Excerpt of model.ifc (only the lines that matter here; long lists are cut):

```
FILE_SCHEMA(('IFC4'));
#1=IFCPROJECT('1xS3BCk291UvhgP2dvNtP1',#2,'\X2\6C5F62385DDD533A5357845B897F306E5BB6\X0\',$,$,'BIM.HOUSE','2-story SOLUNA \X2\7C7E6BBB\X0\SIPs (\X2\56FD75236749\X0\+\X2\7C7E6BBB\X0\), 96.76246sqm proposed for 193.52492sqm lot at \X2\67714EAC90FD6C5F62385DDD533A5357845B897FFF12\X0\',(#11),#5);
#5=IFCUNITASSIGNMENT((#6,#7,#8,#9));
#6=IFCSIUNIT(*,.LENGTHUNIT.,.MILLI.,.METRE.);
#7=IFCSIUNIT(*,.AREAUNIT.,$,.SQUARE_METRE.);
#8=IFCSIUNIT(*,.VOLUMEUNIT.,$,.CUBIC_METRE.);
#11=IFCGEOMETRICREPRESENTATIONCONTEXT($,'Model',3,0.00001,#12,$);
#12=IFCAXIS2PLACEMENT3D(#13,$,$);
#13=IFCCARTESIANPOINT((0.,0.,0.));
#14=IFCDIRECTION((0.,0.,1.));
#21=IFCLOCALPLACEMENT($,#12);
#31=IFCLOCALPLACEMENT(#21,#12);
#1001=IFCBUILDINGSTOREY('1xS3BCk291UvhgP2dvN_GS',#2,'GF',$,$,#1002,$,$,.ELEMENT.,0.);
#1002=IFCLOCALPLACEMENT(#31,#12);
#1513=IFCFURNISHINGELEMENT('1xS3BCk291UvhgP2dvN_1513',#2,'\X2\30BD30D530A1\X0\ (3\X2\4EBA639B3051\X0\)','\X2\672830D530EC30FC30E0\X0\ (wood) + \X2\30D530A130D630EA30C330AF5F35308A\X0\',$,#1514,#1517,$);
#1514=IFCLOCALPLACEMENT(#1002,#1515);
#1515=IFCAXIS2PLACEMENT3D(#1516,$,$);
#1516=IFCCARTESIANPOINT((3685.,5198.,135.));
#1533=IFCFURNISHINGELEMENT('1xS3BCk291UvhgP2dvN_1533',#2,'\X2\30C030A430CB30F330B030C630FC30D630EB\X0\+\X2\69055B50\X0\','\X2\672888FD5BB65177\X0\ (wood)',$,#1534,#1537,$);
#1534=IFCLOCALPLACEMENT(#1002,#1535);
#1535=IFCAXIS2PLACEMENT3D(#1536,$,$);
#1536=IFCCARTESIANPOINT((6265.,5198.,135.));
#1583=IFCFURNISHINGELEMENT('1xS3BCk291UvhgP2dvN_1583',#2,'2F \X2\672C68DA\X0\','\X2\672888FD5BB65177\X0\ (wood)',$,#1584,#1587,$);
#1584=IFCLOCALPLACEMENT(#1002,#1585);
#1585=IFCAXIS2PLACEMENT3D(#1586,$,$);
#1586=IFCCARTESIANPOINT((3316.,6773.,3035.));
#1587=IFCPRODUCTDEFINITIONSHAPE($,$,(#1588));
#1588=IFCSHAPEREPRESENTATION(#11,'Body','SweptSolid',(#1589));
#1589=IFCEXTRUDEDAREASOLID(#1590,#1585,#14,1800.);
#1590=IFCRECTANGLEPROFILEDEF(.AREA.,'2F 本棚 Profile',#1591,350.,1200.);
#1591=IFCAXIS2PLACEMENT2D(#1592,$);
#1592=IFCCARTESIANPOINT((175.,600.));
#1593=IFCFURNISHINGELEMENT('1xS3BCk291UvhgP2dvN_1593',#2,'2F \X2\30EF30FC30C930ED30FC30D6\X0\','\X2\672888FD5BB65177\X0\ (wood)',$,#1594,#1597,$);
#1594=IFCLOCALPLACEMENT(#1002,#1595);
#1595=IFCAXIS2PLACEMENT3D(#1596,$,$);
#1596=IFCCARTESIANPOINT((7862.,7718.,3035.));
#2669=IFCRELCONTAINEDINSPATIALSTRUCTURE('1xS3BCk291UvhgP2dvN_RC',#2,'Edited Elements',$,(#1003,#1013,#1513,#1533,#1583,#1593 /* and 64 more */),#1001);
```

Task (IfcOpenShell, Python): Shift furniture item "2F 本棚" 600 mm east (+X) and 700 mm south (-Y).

```python
import ifcopenshell
import ifcopenshell.api.geometry
import ifcopenshell.util.placement

model = ifcopenshell.open("model.ifc")

item = model.by_id(1583)
matrix = ifcopenshell.util.placement.get_local_placement(item.ObjectPlacement)
matrix[0, 3] += 600.0
matrix[1, 3] -= 700.0
ifcopenshell.api.geometry.edit_object_placement(model, product=item, matrix=matrix, is_si=False)

print(ifcopenshell.util.placement.get_local_placement(item.ObjectPlacement).round(3) + 0.0)

model.write("model_updated.ifc")
```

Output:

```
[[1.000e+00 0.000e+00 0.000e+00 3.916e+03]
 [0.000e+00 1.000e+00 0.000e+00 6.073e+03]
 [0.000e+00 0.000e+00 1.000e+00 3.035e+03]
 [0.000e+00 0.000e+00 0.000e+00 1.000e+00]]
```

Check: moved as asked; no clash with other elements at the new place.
